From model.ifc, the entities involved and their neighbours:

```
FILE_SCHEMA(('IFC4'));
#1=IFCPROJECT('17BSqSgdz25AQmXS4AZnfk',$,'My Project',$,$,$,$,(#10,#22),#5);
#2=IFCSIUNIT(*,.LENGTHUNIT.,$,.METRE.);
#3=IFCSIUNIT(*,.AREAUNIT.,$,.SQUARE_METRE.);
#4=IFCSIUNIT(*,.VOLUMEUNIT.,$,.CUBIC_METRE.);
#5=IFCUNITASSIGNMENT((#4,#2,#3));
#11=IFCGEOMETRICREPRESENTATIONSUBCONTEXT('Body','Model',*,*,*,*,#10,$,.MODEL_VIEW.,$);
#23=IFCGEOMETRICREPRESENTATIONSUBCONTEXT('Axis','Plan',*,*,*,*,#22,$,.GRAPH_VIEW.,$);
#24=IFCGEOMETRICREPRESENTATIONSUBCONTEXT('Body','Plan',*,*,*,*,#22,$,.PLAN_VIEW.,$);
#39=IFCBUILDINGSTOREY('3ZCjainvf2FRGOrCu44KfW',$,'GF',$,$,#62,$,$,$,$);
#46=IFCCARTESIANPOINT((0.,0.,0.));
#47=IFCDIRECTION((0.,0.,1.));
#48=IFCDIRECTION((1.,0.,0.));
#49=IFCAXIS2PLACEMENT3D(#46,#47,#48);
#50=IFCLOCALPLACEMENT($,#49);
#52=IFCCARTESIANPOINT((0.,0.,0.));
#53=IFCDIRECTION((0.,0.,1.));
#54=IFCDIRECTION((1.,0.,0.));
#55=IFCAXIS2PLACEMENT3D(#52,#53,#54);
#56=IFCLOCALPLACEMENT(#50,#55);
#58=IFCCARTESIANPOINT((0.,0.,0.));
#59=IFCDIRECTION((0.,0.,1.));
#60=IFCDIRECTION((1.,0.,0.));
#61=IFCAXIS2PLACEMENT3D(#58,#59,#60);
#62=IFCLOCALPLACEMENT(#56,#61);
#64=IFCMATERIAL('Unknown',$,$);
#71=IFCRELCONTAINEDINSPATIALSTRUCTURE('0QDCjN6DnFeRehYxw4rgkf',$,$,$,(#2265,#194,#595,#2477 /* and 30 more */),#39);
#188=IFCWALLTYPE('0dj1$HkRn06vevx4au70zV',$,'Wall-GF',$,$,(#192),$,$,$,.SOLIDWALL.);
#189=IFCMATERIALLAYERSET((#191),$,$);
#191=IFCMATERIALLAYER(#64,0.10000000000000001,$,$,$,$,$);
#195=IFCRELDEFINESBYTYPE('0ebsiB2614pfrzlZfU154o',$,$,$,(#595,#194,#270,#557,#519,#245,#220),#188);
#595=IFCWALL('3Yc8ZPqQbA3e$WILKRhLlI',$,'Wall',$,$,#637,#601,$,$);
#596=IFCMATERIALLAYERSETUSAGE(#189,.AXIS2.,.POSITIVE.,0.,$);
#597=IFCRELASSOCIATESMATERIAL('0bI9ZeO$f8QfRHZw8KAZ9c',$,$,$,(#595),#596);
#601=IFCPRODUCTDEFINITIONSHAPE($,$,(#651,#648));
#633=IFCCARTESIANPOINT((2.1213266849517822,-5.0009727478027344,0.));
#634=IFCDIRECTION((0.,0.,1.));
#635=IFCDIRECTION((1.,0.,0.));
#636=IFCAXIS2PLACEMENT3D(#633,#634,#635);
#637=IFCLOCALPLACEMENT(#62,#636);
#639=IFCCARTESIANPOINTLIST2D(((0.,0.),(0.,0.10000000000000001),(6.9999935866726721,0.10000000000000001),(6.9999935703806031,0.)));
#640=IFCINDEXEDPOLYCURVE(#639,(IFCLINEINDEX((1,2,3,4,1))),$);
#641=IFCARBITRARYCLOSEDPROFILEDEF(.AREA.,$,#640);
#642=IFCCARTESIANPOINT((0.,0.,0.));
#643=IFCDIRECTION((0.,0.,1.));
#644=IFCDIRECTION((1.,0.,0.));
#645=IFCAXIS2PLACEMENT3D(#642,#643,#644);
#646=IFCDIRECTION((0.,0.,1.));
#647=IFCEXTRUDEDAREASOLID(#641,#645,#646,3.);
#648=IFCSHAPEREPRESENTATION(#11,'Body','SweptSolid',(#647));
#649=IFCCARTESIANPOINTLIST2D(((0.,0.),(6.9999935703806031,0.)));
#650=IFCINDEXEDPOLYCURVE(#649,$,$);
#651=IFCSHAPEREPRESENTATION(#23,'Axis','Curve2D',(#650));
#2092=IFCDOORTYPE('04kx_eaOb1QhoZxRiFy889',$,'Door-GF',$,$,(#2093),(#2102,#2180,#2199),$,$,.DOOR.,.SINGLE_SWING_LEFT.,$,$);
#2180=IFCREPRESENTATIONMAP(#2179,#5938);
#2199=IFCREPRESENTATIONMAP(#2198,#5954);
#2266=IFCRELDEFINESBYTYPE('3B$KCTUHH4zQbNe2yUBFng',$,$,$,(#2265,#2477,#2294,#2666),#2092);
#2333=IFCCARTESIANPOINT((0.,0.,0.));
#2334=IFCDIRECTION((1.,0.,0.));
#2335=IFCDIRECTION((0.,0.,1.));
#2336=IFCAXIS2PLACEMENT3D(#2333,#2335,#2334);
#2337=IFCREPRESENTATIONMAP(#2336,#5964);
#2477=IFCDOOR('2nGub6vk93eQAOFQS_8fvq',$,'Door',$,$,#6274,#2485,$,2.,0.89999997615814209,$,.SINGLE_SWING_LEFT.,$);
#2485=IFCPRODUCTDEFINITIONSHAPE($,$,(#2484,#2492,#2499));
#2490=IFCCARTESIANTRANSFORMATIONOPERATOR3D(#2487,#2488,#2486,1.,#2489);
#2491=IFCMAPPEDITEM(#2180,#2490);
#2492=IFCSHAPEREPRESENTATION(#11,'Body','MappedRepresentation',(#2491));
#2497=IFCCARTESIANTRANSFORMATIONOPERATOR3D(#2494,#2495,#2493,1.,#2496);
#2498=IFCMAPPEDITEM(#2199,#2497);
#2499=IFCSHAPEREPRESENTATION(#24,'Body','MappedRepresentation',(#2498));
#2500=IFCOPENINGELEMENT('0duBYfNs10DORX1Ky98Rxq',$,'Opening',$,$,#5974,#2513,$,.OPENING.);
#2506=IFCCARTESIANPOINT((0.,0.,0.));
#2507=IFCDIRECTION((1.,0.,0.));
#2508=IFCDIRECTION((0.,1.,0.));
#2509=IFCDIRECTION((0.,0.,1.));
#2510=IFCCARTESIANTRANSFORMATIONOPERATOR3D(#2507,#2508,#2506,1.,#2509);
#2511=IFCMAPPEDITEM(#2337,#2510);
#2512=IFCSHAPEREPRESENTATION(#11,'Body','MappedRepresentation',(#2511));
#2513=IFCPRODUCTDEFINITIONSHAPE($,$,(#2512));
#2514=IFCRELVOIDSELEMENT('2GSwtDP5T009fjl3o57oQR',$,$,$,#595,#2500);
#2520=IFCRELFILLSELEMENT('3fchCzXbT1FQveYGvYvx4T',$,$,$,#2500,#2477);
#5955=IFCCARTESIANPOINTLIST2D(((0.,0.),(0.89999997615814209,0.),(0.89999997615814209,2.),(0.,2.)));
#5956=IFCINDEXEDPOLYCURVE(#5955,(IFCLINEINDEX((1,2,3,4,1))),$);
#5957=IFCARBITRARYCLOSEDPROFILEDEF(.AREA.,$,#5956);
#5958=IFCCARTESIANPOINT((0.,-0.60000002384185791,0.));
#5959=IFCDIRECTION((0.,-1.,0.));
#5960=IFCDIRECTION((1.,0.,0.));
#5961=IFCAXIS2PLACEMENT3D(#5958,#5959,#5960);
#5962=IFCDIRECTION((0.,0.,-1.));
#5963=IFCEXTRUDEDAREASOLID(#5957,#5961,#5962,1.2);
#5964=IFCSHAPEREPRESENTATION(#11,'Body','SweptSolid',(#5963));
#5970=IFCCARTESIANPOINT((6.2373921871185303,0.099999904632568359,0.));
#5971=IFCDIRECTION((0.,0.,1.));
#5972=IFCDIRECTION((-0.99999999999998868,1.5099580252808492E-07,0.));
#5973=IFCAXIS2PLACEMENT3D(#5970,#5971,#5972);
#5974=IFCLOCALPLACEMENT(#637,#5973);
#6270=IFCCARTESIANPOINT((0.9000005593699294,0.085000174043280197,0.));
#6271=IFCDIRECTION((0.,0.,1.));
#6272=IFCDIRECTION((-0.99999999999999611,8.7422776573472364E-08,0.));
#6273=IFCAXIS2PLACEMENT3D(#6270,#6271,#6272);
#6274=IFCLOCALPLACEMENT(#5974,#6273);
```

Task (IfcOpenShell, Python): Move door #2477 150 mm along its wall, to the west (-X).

```python
import ifcopenshell
import ifcopenshell.api.geometry
import ifcopenshell.util.placement
import ifcopenshell.util.unit

model = ifcopenshell.open("model.ifc")
unit_scale = ifcopenshell.util.unit.calculate_unit_scale(model)

door = model.by_guid("2nGub6vk93eQAOFQS_8fvq")
opening = door.FillsVoids[0].RelatingOpeningElement
wall = opening.VoidsElements[0].RelatingBuildingElement

wall_matrix = ifcopenshell.util.placement.get_local_placement(wall.ObjectPlacement)
shift = wall_matrix[:3, 0] * -0.15 / unit_scale
before = ifcopenshell.util.placement.get_local_placement(door.ObjectPlacement)[:3, 3].copy()

# The door is placed relative to its opening, so it follows when the opening moves.
matrix = ifcopenshell.util.placement.get_local_placement(opening.ObjectPlacement)
matrix[:3, 3] += shift
ifcopenshell.api.geometry.edit_object_placement(
    model, product=opening, matrix=matrix, is_si=False, should_transform_children=True
)

after = ifcopenshell.util.placement.get_local_placement(door.ObjectPlacement)[:3, 3]
print("door moved by", (after - before).round(3) + 0.0)

model.write("model_v2.ifc")
```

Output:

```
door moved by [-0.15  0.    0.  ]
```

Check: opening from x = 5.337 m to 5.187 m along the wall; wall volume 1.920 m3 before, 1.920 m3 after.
